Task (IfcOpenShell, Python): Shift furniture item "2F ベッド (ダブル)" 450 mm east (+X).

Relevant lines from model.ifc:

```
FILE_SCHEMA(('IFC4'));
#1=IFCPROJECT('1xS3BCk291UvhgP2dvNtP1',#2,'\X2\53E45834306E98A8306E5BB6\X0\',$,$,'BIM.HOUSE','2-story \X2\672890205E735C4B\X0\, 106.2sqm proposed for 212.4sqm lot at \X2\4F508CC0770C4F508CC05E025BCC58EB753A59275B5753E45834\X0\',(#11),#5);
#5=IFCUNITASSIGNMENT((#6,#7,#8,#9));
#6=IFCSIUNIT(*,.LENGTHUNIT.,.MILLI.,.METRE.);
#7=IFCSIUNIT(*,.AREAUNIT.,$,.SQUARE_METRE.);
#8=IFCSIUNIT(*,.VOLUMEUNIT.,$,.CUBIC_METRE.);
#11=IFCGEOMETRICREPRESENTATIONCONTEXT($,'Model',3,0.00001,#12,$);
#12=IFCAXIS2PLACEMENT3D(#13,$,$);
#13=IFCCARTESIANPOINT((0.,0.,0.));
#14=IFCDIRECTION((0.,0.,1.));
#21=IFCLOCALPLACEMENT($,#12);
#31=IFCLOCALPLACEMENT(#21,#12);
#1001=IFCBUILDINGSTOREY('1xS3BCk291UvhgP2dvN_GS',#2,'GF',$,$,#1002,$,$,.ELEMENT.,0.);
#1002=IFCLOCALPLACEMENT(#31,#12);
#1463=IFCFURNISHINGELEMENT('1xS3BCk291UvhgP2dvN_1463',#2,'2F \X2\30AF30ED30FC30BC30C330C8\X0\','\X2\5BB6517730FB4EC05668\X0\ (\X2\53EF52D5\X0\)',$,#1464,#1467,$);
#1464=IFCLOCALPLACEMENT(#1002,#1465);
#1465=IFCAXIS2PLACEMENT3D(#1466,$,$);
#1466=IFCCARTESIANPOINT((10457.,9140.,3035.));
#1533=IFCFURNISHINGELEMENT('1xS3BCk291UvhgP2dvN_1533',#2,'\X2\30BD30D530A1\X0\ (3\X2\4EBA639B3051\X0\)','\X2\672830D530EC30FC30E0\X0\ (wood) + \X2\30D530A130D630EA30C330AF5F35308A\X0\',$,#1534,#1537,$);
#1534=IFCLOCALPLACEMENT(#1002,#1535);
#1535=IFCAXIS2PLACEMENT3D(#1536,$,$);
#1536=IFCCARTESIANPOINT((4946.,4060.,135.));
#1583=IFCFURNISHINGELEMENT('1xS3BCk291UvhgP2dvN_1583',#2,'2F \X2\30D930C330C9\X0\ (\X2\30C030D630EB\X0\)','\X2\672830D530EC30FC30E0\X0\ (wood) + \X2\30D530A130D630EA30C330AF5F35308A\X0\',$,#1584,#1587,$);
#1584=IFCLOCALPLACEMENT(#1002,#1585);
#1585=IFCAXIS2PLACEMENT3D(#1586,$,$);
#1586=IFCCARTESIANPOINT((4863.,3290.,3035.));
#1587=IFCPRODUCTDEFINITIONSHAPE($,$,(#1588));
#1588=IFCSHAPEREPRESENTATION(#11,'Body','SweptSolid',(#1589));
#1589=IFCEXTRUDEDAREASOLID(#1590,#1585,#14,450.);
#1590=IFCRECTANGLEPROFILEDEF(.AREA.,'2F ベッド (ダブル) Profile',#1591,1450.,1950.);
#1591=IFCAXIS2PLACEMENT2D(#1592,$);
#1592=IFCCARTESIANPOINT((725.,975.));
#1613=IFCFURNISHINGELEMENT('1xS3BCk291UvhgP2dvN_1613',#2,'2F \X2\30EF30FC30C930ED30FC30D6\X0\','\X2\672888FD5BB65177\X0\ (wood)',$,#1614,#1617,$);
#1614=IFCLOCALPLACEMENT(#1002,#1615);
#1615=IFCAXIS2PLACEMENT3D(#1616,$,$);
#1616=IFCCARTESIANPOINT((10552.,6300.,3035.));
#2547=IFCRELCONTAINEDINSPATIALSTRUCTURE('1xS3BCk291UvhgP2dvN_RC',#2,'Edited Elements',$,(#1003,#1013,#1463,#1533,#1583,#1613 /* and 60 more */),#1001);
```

```python
import ifcopenshell
import ifcopenshell.api.geometry
import ifcopenshell.util.placement

model = ifcopenshell.open("model.ifc")

item = model.by_guid("1xS3BCk291UvhgP2dvN_1583")
matrix = ifcopenshell.util.placement.get_local_placement(item.ObjectPlacement)
matrix[0, 3] += 450.0
ifcopenshell.api.geometry.edit_object_placement(model, product=item, matrix=matrix, is_si=False)

print(ifcopenshell.util.placement.get_local_placement(item.ObjectPlacement).round(3) + 0.0)

model.write("model_rev.ifc")
```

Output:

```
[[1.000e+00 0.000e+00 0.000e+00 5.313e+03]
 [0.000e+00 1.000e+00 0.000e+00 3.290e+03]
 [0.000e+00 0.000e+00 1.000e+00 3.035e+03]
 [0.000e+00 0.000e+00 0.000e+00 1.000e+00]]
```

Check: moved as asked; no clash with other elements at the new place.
